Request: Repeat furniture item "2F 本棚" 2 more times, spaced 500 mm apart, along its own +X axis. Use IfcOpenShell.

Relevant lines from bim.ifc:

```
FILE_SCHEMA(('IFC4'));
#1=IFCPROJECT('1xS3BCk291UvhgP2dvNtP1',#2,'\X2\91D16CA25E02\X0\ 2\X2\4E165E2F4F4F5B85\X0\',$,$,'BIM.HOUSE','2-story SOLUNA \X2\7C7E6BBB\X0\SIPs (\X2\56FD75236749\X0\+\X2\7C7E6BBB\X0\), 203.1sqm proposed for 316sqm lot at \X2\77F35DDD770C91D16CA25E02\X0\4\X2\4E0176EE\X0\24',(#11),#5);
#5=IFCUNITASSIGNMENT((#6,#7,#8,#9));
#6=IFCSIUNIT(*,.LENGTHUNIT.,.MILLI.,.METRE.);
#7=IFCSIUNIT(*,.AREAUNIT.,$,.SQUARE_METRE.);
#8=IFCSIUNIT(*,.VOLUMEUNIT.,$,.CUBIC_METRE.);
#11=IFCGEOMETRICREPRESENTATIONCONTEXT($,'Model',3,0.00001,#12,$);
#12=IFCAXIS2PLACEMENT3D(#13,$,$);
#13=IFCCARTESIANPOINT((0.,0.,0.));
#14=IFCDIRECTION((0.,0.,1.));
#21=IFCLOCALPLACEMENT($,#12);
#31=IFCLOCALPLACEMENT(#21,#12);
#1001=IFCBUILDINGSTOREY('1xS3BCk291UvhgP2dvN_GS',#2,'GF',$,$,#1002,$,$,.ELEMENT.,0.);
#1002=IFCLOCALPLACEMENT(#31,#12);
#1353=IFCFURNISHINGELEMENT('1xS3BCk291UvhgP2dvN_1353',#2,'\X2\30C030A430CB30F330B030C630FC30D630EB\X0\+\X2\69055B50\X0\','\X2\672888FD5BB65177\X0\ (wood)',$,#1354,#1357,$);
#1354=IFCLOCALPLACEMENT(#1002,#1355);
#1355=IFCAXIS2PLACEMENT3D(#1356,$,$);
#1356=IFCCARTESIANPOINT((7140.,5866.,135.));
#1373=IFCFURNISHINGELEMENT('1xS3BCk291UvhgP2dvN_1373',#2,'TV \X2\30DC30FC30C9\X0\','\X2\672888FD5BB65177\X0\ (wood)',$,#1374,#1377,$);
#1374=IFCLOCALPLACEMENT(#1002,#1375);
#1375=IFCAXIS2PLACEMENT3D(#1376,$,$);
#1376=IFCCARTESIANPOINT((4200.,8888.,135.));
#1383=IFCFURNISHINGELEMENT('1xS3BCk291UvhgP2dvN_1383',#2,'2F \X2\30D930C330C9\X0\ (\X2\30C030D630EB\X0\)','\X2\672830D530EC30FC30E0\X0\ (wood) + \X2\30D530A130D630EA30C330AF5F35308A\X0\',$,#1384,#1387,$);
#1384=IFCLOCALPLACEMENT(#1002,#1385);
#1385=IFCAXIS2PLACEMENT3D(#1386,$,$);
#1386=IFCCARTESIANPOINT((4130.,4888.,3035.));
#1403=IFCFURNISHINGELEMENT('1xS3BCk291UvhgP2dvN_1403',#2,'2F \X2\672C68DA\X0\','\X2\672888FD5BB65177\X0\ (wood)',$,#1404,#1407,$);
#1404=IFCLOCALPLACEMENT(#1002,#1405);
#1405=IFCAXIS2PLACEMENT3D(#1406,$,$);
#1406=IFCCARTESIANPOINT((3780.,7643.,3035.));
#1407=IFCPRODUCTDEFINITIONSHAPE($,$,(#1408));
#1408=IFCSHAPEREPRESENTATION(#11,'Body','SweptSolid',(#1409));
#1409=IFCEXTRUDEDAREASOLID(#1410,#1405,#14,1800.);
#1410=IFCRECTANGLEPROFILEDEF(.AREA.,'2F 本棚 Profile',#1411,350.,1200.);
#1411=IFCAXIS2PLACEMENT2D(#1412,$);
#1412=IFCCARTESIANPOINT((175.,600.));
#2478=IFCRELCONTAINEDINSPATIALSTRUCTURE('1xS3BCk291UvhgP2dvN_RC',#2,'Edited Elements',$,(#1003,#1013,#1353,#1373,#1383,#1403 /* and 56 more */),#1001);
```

```python
import ifcopenshell
import ifcopenshell.api.geometry
import ifcopenshell.api.root
import ifcopenshell.util.element
import ifcopenshell.util.placement
import ifcopenshell.util.unit

model = ifcopenshell.open("bim.ifc")
unit_scale = ifcopenshell.util.unit.calculate_unit_scale(model)


def reuse_history(source, copy):
    """copy_class also copies each property set's owner history, people and application; keep the originals."""
    for rel in copy.IsDefinedBy:
        if rel.is_a("IfcRelDefinesByProperties") and (history := rel.RelatingPropertyDefinition.OwnerHistory):
            rel.RelatingPropertyDefinition.OwnerHistory = source.OwnerHistory
            ifcopenshell.util.element.remove_deep2(model, history)


source = model.by_id(1403)
base = ifcopenshell.util.placement.get_local_placement(source.ObjectPlacement)
step = base[:3, 0] * 0.5 / unit_scale

for i in range(1, 3):
    copy = ifcopenshell.api.root.copy_class(model, product=source)
    copy.Representation = ifcopenshell.util.element.copy_deep(
        model, source.Representation, exclude=["IfcGeometricRepresentationContext", "IfcRepresentationMap"]
    )
    reuse_history(source, copy)
    matrix = base.copy()
    matrix[:3, 3] += i * step
    print("added at", matrix[:3, 3].round(3) + 0.0)
    ifcopenshell.api.geometry.edit_object_placement(model, product=copy, matrix=matrix, is_si=False)

model.write("bim_edited.ifc")
```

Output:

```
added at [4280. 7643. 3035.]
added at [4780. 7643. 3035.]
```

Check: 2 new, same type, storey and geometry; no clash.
